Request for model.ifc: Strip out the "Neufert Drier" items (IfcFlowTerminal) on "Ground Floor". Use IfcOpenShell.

First a look at what the model holds.

```python
import ifcopenshell
import ifcopenshell.util.element

model = ifcopenshell.open("model.ifc")
print(model.schema)
storey = next(s for s in model.by_type("IfcBuildingStorey") if s.Name == "Ground Floor")
terminals = [e for e in ifcopenshell.util.element.get_decomposition(storey) if e.is_a("IfcFlowTerminal")]
seen = {}
for e in terminals:
    element_type = ifcopenshell.util.element.get_type(e)
    name = element_type.Name if element_type not in (None, e) else None
    seen[name] = seen.get(name, 0) + 1
for name, count in sorted(seen.items(), key=str):
    print(count, "x", name)
```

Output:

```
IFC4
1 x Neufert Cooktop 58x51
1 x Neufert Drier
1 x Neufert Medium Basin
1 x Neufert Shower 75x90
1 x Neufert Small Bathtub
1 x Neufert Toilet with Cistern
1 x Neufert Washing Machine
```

```python
import ifcopenshell
import ifcopenshell.api.root
import ifcopenshell.util.element

model = ifcopenshell.open("model.ifc")

storey = next(s for s in model.by_type("IfcBuildingStorey") if s.Name == "Ground Floor")
terminals = [e for e in ifcopenshell.util.element.get_decomposition(storey) if e.is_a("IfcFlowTerminal")]
targets = [e for e in terminals if (t := ifcopenshell.util.element.get_type(e)) not in (None, e) and t.Name == "Neufert Drier"]

for e in targets:
    ifcopenshell.api.root.remove_product(model, product=e)
print(len(targets), "removed")

model.write("model_v2.ifc")
```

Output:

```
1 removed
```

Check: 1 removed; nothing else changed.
